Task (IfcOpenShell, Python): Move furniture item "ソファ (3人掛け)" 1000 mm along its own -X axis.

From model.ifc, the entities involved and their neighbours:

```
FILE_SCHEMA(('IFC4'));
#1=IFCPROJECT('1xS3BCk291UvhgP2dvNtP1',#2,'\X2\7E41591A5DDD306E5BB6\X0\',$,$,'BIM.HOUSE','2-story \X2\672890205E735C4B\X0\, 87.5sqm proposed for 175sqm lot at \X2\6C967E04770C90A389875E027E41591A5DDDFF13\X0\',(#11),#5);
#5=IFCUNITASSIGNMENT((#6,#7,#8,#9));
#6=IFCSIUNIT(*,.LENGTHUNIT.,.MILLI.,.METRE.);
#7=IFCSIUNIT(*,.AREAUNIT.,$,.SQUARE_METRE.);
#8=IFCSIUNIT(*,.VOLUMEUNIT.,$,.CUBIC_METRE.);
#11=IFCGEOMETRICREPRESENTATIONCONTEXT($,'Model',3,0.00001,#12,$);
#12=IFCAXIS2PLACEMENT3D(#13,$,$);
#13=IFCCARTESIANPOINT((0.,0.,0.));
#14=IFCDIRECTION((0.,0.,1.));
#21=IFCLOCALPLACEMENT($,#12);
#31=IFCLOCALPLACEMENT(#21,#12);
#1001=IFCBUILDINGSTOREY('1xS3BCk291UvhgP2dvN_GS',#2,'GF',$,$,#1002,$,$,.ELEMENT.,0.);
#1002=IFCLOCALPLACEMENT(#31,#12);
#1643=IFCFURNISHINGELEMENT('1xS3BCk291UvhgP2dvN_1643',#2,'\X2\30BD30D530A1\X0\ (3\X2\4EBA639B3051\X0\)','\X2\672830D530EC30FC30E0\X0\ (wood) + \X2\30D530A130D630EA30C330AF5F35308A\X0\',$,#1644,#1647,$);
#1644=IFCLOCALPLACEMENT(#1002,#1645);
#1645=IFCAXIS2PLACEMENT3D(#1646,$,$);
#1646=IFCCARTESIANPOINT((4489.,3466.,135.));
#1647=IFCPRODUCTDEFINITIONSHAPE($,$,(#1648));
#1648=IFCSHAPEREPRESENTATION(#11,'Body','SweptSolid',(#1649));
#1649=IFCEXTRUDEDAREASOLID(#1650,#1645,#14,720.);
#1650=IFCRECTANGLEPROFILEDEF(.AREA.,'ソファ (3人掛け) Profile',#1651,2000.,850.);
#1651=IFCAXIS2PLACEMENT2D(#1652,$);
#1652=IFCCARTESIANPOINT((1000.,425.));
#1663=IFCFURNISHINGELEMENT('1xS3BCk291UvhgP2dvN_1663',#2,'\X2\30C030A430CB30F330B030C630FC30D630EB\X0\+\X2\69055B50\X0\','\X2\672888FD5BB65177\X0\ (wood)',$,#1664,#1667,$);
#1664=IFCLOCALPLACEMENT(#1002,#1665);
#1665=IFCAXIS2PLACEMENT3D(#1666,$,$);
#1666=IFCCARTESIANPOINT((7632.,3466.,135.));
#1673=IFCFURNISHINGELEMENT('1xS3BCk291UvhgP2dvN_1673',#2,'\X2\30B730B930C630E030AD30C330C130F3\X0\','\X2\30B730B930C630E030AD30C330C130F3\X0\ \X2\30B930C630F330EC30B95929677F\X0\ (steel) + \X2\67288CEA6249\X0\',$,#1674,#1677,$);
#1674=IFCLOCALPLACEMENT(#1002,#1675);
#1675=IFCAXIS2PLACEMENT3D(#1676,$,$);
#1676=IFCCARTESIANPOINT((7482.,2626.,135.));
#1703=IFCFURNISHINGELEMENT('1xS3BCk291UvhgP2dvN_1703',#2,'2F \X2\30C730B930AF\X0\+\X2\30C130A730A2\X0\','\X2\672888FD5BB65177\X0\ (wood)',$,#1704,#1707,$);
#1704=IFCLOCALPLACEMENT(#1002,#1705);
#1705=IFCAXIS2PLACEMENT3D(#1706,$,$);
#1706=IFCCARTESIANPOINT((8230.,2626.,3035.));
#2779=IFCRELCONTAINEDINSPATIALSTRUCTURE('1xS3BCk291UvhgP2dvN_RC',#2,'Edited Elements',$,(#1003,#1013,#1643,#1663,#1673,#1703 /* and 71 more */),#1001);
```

```python
import ifcopenshell
import ifcopenshell.api.geometry
import ifcopenshell.util.placement

model = ifcopenshell.open("model.ifc")

item = model.by_guid("1xS3BCk291UvhgP2dvN_1643")
matrix = ifcopenshell.util.placement.get_local_placement(item.ObjectPlacement)
matrix[:3, 3] -= matrix[:3, 0] * 1000.0
ifcopenshell.api.geometry.edit_object_placement(model, product=item, matrix=matrix, is_si=False)

print(ifcopenshell.util.placement.get_local_placement(item.ObjectPlacement).round(3) + 0.0)

model.write("model_rev.ifc")
```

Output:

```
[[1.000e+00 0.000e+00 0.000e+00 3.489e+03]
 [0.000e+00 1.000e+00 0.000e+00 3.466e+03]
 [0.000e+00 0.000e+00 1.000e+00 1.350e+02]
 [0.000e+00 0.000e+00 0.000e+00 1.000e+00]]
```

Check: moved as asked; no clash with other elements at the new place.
